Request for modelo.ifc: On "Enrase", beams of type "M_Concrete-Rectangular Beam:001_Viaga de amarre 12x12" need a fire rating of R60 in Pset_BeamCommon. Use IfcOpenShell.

First a look at what the model holds.

```python
import ifcopenshell
import ifcopenshell.util.element

model = ifcopenshell.open("modelo.ifc")
print(model.schema)
storey = next(s for s in model.by_type("IfcBuildingStorey") if s.Name == "Enrase")
beams = [e for e in ifcopenshell.util.element.get_decomposition(storey) if e.is_a("IfcBeam")]
seen = {}
for e in beams:
    element_type = ifcopenshell.util.element.get_type(e)
    key = (element_type.Name if element_type != e and element_type else None, ifcopenshell.util.element.get_pset(e, "Pset_BeamCommon", "FireRating"))
    seen[key] = seen.get(key, 0) + 1
for (name, value), count in sorted(seen.items(), key=str):
    print(count, "x", name, "|", value)
```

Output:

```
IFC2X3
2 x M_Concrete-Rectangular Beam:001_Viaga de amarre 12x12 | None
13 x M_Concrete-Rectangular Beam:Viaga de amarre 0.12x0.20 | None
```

```python
import ifcopenshell
import ifcopenshell.api.pset
import ifcopenshell.util.element

model = ifcopenshell.open("modelo.ifc")

storey = next(s for s in model.by_type("IfcBuildingStorey") if s.Name == "Enrase")
beams = [e for e in ifcopenshell.util.element.get_decomposition(storey) if e.is_a("IfcBeam")]

count = 0
for e in beams:
    element_type = ifcopenshell.util.element.get_type(e)
    if element_type in (None, e) or element_type.Name != "M_Concrete-Rectangular Beam:001_Viaga de amarre 12x12":
        continue
    # add_pset returns the element's existing set when there is one.
    pset = ifcopenshell.api.pset.add_pset(model, product=e, name="Pset_BeamCommon")
    ifcopenshell.api.pset.edit_pset(model, pset=pset, properties={"FireRating": "R60"})
    count += 1

print(count, "beams updated")

model.write("modelo-out.ifc")
```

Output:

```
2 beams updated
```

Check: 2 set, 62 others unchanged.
